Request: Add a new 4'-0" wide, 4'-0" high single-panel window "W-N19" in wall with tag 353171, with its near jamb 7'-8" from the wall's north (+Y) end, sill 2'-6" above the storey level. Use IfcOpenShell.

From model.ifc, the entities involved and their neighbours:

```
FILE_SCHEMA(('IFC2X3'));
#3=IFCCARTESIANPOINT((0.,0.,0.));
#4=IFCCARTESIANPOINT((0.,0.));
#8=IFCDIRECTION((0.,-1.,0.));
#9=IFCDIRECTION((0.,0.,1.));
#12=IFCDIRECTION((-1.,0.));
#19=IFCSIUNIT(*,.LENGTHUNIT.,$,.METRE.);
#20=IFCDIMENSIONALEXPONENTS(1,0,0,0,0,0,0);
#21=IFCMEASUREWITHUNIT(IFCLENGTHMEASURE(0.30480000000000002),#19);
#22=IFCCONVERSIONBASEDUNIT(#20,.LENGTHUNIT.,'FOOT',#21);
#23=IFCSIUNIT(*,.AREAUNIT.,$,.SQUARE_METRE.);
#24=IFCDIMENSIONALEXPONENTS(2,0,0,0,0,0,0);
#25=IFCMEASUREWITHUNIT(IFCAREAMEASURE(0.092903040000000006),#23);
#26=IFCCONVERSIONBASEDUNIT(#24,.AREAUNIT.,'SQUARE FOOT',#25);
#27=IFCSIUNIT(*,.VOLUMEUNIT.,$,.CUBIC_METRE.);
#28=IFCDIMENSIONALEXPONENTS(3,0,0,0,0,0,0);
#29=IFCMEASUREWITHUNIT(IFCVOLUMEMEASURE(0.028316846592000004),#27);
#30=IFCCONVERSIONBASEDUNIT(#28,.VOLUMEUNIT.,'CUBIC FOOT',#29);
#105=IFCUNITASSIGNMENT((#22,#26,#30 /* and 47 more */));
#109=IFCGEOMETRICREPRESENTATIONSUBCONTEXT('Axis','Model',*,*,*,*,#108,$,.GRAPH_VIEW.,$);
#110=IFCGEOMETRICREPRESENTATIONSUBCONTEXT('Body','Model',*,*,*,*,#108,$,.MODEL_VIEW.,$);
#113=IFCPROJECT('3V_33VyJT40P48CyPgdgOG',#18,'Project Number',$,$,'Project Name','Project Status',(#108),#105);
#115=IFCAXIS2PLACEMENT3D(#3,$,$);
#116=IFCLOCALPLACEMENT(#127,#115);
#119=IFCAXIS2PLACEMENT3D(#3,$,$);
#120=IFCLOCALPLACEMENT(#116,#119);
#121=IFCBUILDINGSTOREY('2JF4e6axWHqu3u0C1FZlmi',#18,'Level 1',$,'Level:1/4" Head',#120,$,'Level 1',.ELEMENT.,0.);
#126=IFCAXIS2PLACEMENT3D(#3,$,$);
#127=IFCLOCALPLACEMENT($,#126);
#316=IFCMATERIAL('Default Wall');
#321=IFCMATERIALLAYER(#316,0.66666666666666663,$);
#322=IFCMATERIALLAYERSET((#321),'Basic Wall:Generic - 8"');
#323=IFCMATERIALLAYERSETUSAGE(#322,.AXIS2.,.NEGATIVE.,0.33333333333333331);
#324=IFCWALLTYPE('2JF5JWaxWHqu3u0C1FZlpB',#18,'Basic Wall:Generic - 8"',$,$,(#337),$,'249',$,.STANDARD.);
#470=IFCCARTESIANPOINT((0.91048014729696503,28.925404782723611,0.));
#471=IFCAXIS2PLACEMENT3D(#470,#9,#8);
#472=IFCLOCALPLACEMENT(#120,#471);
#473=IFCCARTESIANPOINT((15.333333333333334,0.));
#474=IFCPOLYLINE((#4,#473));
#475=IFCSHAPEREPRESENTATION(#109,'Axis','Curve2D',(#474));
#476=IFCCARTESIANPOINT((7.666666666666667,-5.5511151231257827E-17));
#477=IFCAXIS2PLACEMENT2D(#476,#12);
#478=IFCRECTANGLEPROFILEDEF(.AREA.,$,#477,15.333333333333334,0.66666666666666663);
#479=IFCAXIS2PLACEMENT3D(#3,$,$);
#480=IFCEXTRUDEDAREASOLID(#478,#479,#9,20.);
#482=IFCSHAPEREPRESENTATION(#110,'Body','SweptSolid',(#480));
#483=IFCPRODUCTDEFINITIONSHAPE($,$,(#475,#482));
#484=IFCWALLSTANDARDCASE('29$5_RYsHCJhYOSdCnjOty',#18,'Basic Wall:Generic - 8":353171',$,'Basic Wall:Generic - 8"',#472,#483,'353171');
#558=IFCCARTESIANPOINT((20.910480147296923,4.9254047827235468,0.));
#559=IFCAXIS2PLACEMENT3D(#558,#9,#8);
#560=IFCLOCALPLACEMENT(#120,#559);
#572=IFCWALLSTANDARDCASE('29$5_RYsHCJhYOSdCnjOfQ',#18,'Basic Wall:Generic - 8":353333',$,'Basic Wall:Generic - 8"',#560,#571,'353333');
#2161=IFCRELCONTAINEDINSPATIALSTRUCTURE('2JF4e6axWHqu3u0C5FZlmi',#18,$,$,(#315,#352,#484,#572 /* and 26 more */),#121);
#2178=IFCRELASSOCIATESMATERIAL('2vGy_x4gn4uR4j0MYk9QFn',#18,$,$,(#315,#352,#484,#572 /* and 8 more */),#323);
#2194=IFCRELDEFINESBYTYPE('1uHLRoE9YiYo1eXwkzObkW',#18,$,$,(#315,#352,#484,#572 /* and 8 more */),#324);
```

```python
import numpy as np
import ifcopenshell
import ifcopenshell.api.feature
import ifcopenshell.api.geometry
import ifcopenshell.api.root
import ifcopenshell.api.spatial
import ifcopenshell.api.type
import ifcopenshell.geom
import ifcopenshell.util.element
import ifcopenshell.util.placement
import ifcopenshell.util.representation
import ifcopenshell.util.shape
import ifcopenshell.util.unit

model = ifcopenshell.open("model.ifc")
unit_scale = ifcopenshell.util.unit.calculate_unit_scale(model)
settings = ifcopenshell.geom.settings()


def volume(element):
    """Net volume in cubic metres, openings subtracted."""
    shape = ifcopenshell.geom.create_shape(settings, element)
    return ifcopenshell.util.shape.get_volume(shape.geometry)


wall = model.by_guid("29$5_RYsHCJhYOSdCnjOty")
storey = ifcopenshell.util.element.get_container(wall, ifc_class="IfcBuildingStorey")
context = ifcopenshell.util.representation.get_context(model, "Model", "Body", "MODEL_VIEW")
before = volume(wall)

width, height, from_end, sill = 1.2192, 1.2192, 2.3368, 0.762  # metres

# The wall runs along its own X axis, and the end named is its -X end.
wall_shape = ifcopenshell.geom.create_shape(settings, wall)
x, y, z = ifcopenshell.util.shape.get_vertices(wall_shape.geometry).T
start = x.min() + from_end
face, thickness = float(y.min()), float(y.max() - y.min())
wall_matrix = ifcopenshell.util.placement.get_local_placement(wall.ObjectPlacement)
level = ifcopenshell.util.placement.get_local_placement(storey.ObjectPlacement)[2, 3]


def in_wall(x, y):
    """Placement at x, y metres in the wall's axes, at sill height."""
    matrix = wall_matrix.copy()
    matrix[:, 3] = wall_matrix @ np.array([x / unit_scale, y / unit_scale, 0.0, 1.0])
    matrix[2, 3] = level + sill / unit_scale
    return matrix


# Opening: a box that overshoots both wall faces by 50 mm.
opening = ifcopenshell.api.root.create_entity(model, ifc_class="IfcOpeningElement")
box = ifcopenshell.api.geometry.add_wall_representation(
    model, context=context, length=width, height=height, thickness=thickness + 0.1
)
ifcopenshell.api.geometry.assign_representation(model, product=opening, representation=box)
ifcopenshell.api.geometry.edit_object_placement(model, product=opening, matrix=in_wall(start, face - 0.05), is_si=False)
ifcopenshell.api.feature.add_feature(model, feature=opening, element=wall)

window = ifcopenshell.api.root.create_entity(model, ifc_class="IfcWindow", name="W-N19")
window.OverallWidth, window.OverallHeight = width / unit_scale, height / unit_scale
body = ifcopenshell.api.geometry.add_window_representation(
    model,
    context=context,
    overall_width=window.OverallWidth,
    overall_height=window.OverallHeight,
    partition_type="SINGLE_PANEL",
)
ifcopenshell.api.geometry.assign_representation(model, product=window, representation=body)
ifcopenshell.api.spatial.assign_container(model, products=[window], relating_structure=storey)
fills = ifcopenshell.api.feature.add_filling(model, opening=opening, element=window)
fills.OwnerHistory = window.OwnerHistory  # required in IFC2X3

# IFC2X3 keeps the operation on the window style.
style = ifcopenshell.api.root.create_entity(model, ifc_class="IfcWindowStyle", name="W-N19")
style.OperationType, style.ConstructionType = "SINGLE_PANEL", "NOTDEFINED"
style.ParameterTakesPrecedence = style.Sizeable = False
ifcopenshell.api.type.assign_type(model, related_objects=[window], relating_type=style)

# Centre the window in the wall's thickness.
ifcopenshell.api.geometry.edit_object_placement(model, product=window, matrix=in_wall(start, face), is_si=False)
window_shape = ifcopenshell.geom.create_shape(settings, window)
depth = ifcopenshell.util.shape.get_vertices(window_shape.geometry)[:, 1]
offset = face + thickness / 2 - (depth.min() + depth.max()) / 2
ifcopenshell.api.geometry.edit_object_placement(model, product=window, matrix=in_wall(start, offset), is_si=False)

after = volume(wall)

print(f"wall volume {before:.3f} -> {after:.3f} m3")

model.write("model_rev.ifc")
```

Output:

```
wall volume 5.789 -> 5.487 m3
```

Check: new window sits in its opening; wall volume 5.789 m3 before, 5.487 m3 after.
